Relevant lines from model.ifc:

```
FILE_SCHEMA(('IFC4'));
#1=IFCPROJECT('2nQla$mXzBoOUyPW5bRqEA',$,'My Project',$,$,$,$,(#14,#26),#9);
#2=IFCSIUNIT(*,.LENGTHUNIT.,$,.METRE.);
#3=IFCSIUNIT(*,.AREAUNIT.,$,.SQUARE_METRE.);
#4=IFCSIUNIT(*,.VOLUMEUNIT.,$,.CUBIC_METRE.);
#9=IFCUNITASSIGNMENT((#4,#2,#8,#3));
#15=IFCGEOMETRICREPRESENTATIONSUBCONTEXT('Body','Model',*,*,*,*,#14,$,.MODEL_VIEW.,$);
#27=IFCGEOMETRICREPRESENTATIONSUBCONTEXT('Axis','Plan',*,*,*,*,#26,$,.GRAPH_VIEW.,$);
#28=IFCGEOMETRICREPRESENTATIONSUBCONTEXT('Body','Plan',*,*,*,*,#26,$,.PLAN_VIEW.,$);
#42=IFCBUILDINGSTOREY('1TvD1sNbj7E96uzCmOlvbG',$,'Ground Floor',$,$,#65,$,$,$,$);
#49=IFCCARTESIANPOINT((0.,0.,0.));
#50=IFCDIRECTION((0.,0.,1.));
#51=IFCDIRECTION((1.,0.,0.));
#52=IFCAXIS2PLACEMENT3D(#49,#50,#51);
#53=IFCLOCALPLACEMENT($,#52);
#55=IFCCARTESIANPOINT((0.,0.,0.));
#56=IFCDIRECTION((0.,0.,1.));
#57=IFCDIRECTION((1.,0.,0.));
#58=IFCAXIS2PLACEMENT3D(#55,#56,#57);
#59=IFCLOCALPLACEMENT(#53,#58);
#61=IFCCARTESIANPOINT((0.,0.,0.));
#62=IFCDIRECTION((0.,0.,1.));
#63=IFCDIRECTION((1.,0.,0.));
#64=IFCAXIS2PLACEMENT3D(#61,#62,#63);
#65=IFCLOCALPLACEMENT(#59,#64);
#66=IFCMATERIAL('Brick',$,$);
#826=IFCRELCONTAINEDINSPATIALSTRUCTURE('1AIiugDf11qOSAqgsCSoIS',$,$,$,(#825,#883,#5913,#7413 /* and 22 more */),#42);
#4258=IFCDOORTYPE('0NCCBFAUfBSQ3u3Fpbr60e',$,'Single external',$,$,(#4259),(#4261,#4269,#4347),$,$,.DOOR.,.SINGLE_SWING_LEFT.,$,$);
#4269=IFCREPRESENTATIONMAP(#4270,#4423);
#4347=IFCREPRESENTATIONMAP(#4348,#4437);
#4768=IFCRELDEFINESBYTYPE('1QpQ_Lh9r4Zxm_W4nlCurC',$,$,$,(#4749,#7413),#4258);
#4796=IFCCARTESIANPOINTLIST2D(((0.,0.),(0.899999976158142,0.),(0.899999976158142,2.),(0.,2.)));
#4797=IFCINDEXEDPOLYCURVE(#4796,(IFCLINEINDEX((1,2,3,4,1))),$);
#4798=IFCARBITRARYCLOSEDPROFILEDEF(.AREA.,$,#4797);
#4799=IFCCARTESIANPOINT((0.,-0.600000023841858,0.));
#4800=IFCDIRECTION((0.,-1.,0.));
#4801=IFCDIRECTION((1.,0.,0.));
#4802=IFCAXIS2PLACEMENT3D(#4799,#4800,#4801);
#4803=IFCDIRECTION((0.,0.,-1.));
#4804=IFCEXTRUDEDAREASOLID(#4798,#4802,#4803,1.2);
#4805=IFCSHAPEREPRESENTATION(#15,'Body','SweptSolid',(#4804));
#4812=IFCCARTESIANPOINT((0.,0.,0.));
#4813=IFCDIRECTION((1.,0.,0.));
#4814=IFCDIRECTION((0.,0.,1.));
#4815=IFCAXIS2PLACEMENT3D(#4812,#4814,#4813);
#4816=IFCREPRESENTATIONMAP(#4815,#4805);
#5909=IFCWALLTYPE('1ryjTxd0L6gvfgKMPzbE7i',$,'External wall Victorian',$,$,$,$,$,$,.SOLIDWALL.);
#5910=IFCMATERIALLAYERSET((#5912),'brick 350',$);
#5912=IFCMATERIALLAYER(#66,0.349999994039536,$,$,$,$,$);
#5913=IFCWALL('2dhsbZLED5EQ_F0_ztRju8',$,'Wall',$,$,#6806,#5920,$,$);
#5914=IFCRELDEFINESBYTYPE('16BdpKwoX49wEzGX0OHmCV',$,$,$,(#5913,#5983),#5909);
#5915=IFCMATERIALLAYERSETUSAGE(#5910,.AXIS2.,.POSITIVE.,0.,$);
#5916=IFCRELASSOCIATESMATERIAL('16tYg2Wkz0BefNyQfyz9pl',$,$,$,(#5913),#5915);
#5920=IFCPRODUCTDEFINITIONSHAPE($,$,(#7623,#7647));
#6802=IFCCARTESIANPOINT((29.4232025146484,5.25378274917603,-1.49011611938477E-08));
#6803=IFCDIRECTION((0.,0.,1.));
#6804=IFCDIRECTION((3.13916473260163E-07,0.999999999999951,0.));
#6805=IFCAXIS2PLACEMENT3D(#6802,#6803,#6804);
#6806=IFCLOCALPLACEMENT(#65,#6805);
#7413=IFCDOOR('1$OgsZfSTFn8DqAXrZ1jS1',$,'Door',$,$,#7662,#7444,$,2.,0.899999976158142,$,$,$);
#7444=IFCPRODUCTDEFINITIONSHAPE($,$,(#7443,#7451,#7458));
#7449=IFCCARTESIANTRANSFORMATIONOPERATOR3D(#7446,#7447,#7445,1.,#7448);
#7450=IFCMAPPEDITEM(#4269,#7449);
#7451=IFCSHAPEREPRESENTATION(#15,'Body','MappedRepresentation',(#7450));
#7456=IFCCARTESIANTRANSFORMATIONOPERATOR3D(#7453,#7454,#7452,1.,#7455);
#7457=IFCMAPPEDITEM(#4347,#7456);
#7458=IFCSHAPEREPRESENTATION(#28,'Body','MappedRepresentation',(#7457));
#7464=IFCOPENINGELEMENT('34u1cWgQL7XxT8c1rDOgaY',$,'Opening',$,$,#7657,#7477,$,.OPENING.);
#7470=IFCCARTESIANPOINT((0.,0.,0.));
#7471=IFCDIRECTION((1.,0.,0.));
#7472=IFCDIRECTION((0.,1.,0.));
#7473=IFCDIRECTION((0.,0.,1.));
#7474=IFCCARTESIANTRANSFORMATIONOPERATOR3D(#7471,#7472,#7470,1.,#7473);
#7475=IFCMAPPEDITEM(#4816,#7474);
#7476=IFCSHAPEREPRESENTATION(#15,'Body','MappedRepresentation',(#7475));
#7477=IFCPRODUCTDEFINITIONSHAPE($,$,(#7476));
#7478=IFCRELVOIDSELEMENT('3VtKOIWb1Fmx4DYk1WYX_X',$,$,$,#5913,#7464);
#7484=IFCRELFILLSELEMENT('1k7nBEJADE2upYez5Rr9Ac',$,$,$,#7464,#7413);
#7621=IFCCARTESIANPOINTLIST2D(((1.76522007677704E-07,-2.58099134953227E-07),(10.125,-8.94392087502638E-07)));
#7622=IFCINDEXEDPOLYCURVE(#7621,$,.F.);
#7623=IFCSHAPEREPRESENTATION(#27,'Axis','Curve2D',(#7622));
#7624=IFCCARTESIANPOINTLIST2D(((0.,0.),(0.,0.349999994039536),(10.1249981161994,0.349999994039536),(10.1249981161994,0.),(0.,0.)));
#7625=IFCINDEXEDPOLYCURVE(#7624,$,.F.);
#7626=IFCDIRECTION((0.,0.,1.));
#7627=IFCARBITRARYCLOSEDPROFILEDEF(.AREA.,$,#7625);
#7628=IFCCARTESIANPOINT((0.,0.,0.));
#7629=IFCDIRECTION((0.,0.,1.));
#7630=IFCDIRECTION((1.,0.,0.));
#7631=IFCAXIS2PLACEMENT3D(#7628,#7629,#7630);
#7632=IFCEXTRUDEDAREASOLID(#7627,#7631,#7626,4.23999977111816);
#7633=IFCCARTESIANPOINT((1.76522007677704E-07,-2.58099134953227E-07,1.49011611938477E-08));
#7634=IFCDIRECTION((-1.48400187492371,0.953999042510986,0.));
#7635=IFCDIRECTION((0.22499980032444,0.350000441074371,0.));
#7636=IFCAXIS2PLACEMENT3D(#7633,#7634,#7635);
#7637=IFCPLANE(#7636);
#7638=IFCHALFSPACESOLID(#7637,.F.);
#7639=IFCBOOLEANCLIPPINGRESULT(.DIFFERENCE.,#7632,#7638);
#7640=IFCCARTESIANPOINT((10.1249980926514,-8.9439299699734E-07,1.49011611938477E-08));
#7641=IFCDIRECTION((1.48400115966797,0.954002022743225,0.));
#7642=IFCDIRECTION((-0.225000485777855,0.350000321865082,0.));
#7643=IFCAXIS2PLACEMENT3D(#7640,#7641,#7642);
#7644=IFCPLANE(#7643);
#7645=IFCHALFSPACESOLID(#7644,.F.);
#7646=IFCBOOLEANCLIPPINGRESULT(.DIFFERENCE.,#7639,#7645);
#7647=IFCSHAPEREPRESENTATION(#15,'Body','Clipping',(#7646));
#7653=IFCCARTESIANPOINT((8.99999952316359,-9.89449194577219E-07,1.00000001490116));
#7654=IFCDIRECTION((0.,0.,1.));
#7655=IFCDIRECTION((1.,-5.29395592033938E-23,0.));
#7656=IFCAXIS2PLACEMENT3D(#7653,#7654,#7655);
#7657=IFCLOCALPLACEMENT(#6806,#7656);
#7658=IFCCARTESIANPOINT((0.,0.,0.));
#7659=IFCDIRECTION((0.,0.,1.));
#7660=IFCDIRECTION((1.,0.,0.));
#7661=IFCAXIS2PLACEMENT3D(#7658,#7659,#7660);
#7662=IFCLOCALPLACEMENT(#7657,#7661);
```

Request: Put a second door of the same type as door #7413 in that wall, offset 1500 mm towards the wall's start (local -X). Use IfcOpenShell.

```python
import ifcopenshell
import ifcopenshell.api.feature
import ifcopenshell.api.geometry
import ifcopenshell.api.root
import ifcopenshell.geom
import ifcopenshell.util.element
import ifcopenshell.util.placement
import ifcopenshell.util.shape

model = ifcopenshell.open("model.ifc")
settings = ifcopenshell.geom.settings()


def volume(element):
    """Net volume in cubic metres, openings subtracted."""
    shape = ifcopenshell.geom.create_shape(settings, element)
    return ifcopenshell.util.shape.get_volume(shape.geometry)


door = model.by_id(7413)
opening = door.FillsVoids[0].RelatingOpeningElement
wall = opening.VoidsElements[0].RelatingBuildingElement
before = volume(wall)
shift = ifcopenshell.util.placement.get_local_placement(wall.ObjectPlacement)[:3, 0] * -1.5

# copy_class copies the void relationship, type, container and properties, but no geometry.
new_opening = ifcopenshell.api.root.copy_class(model, product=opening)
new_opening.Representation = ifcopenshell.util.element.copy_deep(
    model, opening.Representation, exclude=["IfcGeometricRepresentationContext", "IfcRepresentationMap"]
)
new_door = ifcopenshell.api.root.copy_class(model, product=door)
new_door.Representation = ifcopenshell.util.element.copy_deep(
    model, door.Representation, exclude=["IfcGeometricRepresentationContext", "IfcRepresentationMap"]
)
ifcopenshell.api.feature.add_filling(model, opening=new_opening, element=new_door)

for old, new in ((opening, new_opening), (door, new_door)):
    matrix = ifcopenshell.util.placement.get_local_placement(old.ObjectPlacement)
    matrix[:3, 3] += shift
    ifcopenshell.api.geometry.edit_object_placement(model, product=new, matrix=matrix, is_si=False)

after = volume(wall)

print(f"wall volume {before:.3f} -> {after:.3f} m3")

model.write("model_updated.ifc")
```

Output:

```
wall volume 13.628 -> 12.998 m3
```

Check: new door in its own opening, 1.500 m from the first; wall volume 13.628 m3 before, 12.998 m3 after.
